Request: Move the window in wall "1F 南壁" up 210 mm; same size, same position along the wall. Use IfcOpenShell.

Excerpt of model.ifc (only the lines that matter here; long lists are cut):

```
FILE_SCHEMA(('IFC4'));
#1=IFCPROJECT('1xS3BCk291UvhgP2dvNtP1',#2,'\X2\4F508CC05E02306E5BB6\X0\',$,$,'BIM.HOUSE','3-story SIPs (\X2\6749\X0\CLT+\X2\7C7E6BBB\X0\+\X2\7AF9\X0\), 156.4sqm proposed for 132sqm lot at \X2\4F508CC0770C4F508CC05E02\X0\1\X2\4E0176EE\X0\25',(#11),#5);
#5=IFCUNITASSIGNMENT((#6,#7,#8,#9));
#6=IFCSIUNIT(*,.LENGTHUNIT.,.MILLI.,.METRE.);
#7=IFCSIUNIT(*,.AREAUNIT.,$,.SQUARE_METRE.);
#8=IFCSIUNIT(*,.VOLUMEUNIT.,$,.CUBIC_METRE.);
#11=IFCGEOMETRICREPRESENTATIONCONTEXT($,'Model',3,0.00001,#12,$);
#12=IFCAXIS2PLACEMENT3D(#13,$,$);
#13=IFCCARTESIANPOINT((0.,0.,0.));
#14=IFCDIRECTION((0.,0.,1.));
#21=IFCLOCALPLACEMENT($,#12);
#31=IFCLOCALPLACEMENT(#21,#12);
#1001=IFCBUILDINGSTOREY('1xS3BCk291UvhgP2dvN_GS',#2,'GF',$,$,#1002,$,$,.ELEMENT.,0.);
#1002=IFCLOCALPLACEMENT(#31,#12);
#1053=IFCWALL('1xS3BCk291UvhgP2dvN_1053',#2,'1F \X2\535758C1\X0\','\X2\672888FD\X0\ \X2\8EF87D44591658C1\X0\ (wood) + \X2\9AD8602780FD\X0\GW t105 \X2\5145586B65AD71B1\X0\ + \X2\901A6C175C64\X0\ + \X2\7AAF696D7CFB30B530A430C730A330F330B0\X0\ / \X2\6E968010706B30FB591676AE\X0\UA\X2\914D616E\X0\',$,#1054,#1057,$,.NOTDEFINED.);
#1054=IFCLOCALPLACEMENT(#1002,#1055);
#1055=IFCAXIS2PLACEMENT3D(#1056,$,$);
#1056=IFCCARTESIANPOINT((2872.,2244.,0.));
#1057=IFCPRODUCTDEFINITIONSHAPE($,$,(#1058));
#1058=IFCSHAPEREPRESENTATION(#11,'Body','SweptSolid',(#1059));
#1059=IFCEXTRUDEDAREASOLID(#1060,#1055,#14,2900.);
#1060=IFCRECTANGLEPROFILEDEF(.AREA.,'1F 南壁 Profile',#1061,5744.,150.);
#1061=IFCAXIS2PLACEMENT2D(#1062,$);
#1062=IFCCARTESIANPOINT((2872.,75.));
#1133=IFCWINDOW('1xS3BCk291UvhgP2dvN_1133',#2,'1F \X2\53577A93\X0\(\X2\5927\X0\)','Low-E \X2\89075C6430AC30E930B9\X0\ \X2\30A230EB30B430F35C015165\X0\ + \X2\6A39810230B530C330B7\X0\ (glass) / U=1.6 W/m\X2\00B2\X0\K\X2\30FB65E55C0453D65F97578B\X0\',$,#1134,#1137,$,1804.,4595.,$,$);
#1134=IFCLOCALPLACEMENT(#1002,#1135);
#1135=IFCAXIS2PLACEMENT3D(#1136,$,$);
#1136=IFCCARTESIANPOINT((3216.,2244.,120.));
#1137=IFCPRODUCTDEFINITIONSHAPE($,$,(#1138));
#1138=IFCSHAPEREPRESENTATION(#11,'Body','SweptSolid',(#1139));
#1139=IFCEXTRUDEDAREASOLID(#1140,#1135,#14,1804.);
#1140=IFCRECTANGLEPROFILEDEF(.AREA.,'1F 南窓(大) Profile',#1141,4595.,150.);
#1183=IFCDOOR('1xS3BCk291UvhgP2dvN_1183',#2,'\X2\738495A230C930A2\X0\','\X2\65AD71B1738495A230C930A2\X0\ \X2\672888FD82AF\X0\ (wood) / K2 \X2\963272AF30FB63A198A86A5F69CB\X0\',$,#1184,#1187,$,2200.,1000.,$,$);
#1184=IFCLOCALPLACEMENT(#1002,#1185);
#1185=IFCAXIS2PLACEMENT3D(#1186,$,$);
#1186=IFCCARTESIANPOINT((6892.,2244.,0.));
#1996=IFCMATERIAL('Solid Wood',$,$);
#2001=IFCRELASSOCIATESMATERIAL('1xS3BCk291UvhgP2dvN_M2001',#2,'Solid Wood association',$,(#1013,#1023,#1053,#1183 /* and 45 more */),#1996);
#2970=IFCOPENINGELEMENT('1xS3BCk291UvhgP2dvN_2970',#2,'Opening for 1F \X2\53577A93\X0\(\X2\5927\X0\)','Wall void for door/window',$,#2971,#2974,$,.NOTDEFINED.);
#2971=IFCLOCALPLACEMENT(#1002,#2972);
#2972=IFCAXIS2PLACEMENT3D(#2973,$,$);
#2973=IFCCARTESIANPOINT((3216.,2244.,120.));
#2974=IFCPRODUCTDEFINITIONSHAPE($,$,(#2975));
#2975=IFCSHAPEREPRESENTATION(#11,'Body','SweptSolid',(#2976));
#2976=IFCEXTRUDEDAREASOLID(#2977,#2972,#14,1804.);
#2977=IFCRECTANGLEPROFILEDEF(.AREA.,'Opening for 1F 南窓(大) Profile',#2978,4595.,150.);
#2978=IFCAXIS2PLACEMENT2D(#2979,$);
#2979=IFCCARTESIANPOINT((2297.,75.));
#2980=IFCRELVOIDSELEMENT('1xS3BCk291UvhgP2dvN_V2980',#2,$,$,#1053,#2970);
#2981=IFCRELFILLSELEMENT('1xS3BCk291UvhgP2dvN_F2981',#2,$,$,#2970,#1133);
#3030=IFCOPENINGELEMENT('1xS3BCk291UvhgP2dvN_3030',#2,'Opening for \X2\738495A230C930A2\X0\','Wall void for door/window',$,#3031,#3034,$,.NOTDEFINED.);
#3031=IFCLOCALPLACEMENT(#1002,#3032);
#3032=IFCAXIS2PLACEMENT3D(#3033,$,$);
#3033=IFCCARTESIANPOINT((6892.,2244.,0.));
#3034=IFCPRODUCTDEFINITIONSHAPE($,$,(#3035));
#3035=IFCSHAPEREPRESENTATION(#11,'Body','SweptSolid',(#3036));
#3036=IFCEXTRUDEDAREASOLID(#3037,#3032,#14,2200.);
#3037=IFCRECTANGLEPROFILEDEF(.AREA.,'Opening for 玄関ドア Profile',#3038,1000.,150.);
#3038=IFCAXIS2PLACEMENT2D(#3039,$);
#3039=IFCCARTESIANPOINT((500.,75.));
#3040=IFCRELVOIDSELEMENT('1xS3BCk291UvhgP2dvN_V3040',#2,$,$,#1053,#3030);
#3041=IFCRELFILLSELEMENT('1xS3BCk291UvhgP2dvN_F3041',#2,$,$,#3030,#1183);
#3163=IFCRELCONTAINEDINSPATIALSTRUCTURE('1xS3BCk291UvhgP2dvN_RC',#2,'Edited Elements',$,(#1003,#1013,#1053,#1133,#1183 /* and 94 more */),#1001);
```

```python
import numpy as np
import ifcopenshell
import ifcopenshell.api.geometry
import ifcopenshell.util.placement
import ifcopenshell.util.unit

model = ifcopenshell.open("model.ifc")
unit_scale = ifcopenshell.util.unit.calculate_unit_scale(model)

window = model.by_guid("1xS3BCk291UvhgP2dvN_1133")
opening = window.FillsVoids[0].RelatingOpeningElement
dz = 0.21 / unit_scale

shift = np.array([0.0, 0.0, dz])
# The window is not placed relative to its opening, so move both.
for product in (opening, window):
    matrix = ifcopenshell.util.placement.get_local_placement(product.ObjectPlacement)
    matrix[:3, 3] += shift
    ifcopenshell.api.geometry.edit_object_placement(model, product=product, matrix=matrix, is_si=False)

print(f"moved by {dz * unit_scale:+.3f} m")

model.write("model_rev.ifc")
```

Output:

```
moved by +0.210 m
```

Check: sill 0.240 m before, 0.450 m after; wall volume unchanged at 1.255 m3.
